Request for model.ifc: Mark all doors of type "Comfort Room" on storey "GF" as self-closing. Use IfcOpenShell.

First a look at what the model holds.

```python
import ifcopenshell
import ifcopenshell.util.element

model = ifcopenshell.open("model.ifc")
print(model.schema)
storey = next(s for s in model.by_type("IfcBuildingStorey") if s.Name == "GF")
doors = [e for e in ifcopenshell.util.element.get_decomposition(storey) if e.is_a("IfcDoor")]
seen = {}
for e in doors:
    element_type = ifcopenshell.util.element.get_type(e)
    key = (element_type.Name if element_type != e and element_type else None, ifcopenshell.util.element.get_pset(e, "Pset_DoorCommon", "SelfClosing"))
    seen[key] = seen.get(key, 0) + 1
for (name, value), count in sorted(seen.items(), key=str):
    print(count, "x", name, "|", value)
```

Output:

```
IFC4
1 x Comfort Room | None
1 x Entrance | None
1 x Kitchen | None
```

```python
import ifcopenshell
import ifcopenshell.api.pset
import ifcopenshell.util.element

model = ifcopenshell.open("model.ifc")

storey = next(s for s in model.by_type("IfcBuildingStorey") if s.Name == "GF")
doors = [e for e in ifcopenshell.util.element.get_decomposition(storey) if e.is_a("IfcDoor")]

count = 0
for e in doors:
    element_type = ifcopenshell.util.element.get_type(e)
    if element_type in (None, e) or element_type.Name != "Comfort Room":
        continue
    # add_pset returns the element's existing set when there is one.
    pset = ifcopenshell.api.pset.add_pset(model, product=e, name="Pset_DoorCommon")
    ifcopenshell.api.pset.edit_pset(model, pset=pset, properties={"SelfClosing": True})
    count += 1

print(count, "doors updated")

model.write("model_edited.ifc")
```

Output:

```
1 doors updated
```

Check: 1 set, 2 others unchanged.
